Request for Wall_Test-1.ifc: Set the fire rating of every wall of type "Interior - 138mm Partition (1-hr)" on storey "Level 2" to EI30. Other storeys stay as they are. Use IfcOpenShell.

First a look at what the model holds.

```python
import ifcopenshell
import ifcopenshell.util.element

model = ifcopenshell.open("Wall_Test-1.ifc")
print(model.schema)
storey = next(s for s in model.by_type("IfcBuildingStorey") if s.Name == "Level 2")
walls = [e for e in ifcopenshell.util.element.get_decomposition(storey) if e.is_a("IfcWall")]
seen = {}
for e in walls:
    element_type = ifcopenshell.util.element.get_type(e)
    key = (element_type.Name if element_type != e and element_type else None, ifcopenshell.util.element.get_pset(e, "Pset_WallCommon", "FireRating"))
    seen[key] = seen.get(key, 0) + 1
for (name, value), count in sorted(seen.items(), key=str):
    print(count, "x", name, "|", value)
```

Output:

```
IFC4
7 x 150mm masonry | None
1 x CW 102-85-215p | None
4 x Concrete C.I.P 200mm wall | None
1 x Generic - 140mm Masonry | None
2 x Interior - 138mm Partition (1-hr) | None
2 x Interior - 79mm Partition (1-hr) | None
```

```python
import ifcopenshell
import ifcopenshell.api.pset
import ifcopenshell.util.element

model = ifcopenshell.open("Wall_Test-1.ifc")

storey = next(s for s in model.by_type("IfcBuildingStorey") if s.Name == "Level 2")
walls = [e for e in ifcopenshell.util.element.get_decomposition(storey) if e.is_a("IfcWall")]

count = 0
for e in walls:
    element_type = ifcopenshell.util.element.get_type(e)
    if element_type in (None, e) or element_type.Name != "Interior - 138mm Partition (1-hr)":
        continue
    # add_pset returns the element's existing set when there is one.
    pset = ifcopenshell.api.pset.add_pset(model, product=e, name="Pset_WallCommon")
    ifcopenshell.api.pset.edit_pset(model, pset=pset, properties={"FireRating": "EI30"})
    count += 1

print(count, "walls updated")

model.write("Wall_Test-1-out.ifc")
```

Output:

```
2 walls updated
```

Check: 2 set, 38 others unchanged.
